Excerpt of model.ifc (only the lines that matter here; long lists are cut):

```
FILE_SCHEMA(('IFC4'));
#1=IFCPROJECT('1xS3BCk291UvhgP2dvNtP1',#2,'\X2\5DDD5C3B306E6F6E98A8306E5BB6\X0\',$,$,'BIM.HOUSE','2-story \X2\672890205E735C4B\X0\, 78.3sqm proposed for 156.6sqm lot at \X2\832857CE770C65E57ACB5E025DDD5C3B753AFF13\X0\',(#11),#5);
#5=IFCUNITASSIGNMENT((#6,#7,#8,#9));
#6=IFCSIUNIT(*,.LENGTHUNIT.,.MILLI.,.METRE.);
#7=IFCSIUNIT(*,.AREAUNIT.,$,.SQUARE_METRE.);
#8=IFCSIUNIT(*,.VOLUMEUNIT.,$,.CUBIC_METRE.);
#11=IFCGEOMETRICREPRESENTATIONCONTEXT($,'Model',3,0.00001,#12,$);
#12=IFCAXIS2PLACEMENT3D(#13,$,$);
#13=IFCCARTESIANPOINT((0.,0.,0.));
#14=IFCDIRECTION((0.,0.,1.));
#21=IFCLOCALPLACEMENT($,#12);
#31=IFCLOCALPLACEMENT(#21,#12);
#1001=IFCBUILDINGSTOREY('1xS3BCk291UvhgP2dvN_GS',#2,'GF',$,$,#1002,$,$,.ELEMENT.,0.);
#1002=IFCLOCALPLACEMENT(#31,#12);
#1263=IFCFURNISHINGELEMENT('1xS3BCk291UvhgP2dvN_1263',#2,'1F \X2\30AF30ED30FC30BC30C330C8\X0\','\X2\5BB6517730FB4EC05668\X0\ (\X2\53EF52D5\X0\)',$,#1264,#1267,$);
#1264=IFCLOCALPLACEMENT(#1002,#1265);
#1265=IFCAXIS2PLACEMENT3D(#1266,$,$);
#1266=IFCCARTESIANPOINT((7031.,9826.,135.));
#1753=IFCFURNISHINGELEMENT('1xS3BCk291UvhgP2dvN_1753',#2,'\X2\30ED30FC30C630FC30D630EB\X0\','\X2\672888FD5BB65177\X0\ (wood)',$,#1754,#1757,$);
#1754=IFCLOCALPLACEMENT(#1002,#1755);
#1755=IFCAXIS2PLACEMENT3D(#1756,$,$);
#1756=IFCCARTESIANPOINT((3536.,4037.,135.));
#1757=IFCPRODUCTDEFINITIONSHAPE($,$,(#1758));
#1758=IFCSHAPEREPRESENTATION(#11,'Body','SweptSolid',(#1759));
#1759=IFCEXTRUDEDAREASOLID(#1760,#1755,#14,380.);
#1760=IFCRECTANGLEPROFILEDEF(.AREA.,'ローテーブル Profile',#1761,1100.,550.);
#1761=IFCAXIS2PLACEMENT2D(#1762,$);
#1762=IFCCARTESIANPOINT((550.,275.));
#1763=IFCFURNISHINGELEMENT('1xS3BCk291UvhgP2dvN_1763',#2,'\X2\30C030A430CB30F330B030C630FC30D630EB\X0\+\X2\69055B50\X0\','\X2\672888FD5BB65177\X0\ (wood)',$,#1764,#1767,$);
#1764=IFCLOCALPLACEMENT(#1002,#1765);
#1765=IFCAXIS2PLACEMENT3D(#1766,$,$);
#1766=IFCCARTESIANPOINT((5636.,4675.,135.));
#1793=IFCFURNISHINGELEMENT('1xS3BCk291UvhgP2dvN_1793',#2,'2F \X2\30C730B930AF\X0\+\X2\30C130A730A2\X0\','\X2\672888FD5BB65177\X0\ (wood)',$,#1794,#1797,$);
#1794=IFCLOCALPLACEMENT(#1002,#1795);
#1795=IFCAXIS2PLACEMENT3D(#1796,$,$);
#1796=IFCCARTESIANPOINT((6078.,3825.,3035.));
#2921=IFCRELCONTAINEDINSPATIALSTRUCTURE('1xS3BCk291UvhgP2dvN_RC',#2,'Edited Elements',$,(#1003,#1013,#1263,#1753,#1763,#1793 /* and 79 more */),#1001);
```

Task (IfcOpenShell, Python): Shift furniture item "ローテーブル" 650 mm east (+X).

```python
import ifcopenshell
import ifcopenshell.api.geometry
import ifcopenshell.util.placement

model = ifcopenshell.open("model.ifc")

item = model.by_guid("1xS3BCk291UvhgP2dvN_1753")
matrix = ifcopenshell.util.placement.get_local_placement(item.ObjectPlacement)
matrix[0, 3] += 650.0
ifcopenshell.api.geometry.edit_object_placement(model, product=item, matrix=matrix, is_si=False)

print(ifcopenshell.util.placement.get_local_placement(item.ObjectPlacement).round(3) + 0.0)

model.write("model-out.ifc")
```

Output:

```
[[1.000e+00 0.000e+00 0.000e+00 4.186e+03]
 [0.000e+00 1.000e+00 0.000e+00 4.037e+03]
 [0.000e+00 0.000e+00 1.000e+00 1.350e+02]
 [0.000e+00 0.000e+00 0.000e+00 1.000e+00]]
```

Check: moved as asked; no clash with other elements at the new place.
